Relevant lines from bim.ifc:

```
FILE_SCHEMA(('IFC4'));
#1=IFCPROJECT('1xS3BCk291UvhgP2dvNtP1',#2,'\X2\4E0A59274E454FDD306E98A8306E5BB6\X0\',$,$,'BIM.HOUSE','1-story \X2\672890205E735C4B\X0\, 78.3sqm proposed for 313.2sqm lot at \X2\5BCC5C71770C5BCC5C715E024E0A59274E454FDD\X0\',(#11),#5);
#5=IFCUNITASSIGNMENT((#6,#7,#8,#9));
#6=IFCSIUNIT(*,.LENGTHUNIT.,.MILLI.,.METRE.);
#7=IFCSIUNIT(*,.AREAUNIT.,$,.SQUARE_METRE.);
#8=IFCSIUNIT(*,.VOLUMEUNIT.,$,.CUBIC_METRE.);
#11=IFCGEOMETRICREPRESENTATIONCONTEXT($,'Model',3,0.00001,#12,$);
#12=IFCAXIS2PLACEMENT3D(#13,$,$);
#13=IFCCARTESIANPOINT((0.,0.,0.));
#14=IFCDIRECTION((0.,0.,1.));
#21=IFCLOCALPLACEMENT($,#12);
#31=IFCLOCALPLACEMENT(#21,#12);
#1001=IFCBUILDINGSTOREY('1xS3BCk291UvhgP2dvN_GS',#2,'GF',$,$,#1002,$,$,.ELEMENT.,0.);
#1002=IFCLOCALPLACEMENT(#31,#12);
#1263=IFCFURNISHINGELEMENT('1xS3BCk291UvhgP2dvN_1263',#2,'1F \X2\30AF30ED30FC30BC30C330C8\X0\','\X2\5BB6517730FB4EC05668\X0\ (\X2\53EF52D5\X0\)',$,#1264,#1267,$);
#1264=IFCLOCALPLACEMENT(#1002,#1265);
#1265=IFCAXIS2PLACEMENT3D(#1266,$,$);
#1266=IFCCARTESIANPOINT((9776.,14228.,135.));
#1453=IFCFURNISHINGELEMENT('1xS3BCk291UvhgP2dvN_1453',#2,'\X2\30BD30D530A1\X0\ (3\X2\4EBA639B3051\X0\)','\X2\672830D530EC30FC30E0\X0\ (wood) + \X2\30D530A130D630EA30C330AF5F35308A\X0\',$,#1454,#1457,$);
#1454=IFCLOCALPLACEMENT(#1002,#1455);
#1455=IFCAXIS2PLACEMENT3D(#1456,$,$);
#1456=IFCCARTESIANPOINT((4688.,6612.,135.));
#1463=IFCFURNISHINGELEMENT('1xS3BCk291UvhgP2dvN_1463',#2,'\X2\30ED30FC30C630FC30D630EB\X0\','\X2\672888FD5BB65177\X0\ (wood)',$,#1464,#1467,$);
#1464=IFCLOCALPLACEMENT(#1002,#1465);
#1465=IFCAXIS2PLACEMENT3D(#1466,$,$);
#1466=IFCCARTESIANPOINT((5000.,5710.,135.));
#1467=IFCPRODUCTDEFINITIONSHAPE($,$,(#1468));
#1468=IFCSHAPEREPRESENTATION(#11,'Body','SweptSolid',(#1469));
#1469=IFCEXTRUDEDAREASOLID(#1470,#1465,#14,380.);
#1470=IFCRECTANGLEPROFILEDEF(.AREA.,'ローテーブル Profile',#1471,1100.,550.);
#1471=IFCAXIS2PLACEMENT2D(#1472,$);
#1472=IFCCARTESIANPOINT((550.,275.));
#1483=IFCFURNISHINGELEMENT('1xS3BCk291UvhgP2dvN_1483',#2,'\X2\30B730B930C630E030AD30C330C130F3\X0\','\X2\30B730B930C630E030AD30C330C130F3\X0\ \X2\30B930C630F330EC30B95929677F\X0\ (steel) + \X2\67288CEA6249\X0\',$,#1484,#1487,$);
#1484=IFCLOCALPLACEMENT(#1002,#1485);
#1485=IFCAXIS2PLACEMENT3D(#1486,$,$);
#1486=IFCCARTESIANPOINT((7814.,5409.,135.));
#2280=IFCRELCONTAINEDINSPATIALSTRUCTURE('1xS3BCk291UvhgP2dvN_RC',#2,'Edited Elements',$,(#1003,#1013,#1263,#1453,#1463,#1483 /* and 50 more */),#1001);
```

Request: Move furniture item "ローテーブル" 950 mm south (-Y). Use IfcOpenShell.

```python
import ifcopenshell
import ifcopenshell.api.geometry
import ifcopenshell.util.placement
import ifcopenshell.util.unit

model = ifcopenshell.open("bim.ifc")
unit_scale = ifcopenshell.util.unit.calculate_unit_scale(model)

item = model.by_guid("1xS3BCk291UvhgP2dvN_1463")
matrix = ifcopenshell.util.placement.get_local_placement(item.ObjectPlacement)
matrix[1, 3] -= 0.95 / unit_scale
ifcopenshell.api.geometry.edit_object_placement(model, product=item, matrix=matrix, is_si=False)

print(ifcopenshell.util.placement.get_local_placement(item.ObjectPlacement).round(3) + 0.0)

model.write("bim_rev.ifc")
```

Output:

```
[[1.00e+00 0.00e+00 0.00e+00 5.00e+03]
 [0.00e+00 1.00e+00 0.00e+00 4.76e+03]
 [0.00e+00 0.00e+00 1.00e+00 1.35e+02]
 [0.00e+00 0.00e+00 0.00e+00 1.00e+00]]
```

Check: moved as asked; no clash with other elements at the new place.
